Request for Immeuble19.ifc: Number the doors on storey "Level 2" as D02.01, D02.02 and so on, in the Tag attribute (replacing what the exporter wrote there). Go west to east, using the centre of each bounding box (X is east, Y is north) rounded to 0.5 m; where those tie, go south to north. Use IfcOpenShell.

First a look at what the model holds.

```python
import ifcopenshell
import ifcopenshell.util.element
import ifcopenshell.util.placement

model = ifcopenshell.open("Immeuble19.ifc")
print(model.schema)
storey = next(s for s in model.by_type("IfcBuildingStorey") if s.Name == "Level 2")
doors = [e for e in ifcopenshell.util.element.get_decomposition(storey) if e.is_a("IfcDoor")]
for e in sorted(doors, key=lambda e: e.id()):
    origin = ifcopenshell.util.placement.get_local_placement(e.ObjectPlacement)[:3, 3]
    print(e.id(), e.Tag, e.Name, origin.round(2) + 0.0, sep=" | ")
```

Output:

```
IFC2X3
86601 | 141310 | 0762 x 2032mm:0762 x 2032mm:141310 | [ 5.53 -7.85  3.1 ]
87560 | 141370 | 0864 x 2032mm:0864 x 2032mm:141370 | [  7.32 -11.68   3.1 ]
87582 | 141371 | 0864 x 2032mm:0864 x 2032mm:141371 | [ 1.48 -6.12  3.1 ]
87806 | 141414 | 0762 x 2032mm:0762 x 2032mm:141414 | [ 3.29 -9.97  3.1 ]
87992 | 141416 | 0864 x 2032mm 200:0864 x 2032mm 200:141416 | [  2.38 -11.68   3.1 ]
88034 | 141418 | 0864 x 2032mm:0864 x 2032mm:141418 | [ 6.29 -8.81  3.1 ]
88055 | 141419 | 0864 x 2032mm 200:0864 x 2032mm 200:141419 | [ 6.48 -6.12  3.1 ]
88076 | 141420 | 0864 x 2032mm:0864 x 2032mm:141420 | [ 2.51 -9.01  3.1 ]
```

```python
import ifcopenshell
import ifcopenshell.geom
import ifcopenshell.util.element
import ifcopenshell.util.shape

model = ifcopenshell.open("Immeuble19.ifc")
settings = ifcopenshell.geom.settings()
settings.set("use-world-coords", True)


def centre(element):
    shape = ifcopenshell.geom.create_shape(settings, element)
    return ifcopenshell.util.shape.get_bbox_centroid(shape.geometry)


storey = next(s for s in model.by_type("IfcBuildingStorey") if s.Name == "Level 2")
doors = [e for e in ifcopenshell.util.element.get_decomposition(storey) if e.is_a("IfcDoor")]

# Insertion points can sit at a corner or the storey origin, so sort by the geometry (in metres).
centres = {e: centre(e) for e in doors}
doors.sort(key=lambda e: (round(centres[e][0] / 0.5), centres[e][1]))

for i, e in enumerate(doors, start=1):
    number = f"D02.{i:02d}"
    e.Tag = number
    print(e.id(), number)

model.write("Immeuble19-out.ifc")
```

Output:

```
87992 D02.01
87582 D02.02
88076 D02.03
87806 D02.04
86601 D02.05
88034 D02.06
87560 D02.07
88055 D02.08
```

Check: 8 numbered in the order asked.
